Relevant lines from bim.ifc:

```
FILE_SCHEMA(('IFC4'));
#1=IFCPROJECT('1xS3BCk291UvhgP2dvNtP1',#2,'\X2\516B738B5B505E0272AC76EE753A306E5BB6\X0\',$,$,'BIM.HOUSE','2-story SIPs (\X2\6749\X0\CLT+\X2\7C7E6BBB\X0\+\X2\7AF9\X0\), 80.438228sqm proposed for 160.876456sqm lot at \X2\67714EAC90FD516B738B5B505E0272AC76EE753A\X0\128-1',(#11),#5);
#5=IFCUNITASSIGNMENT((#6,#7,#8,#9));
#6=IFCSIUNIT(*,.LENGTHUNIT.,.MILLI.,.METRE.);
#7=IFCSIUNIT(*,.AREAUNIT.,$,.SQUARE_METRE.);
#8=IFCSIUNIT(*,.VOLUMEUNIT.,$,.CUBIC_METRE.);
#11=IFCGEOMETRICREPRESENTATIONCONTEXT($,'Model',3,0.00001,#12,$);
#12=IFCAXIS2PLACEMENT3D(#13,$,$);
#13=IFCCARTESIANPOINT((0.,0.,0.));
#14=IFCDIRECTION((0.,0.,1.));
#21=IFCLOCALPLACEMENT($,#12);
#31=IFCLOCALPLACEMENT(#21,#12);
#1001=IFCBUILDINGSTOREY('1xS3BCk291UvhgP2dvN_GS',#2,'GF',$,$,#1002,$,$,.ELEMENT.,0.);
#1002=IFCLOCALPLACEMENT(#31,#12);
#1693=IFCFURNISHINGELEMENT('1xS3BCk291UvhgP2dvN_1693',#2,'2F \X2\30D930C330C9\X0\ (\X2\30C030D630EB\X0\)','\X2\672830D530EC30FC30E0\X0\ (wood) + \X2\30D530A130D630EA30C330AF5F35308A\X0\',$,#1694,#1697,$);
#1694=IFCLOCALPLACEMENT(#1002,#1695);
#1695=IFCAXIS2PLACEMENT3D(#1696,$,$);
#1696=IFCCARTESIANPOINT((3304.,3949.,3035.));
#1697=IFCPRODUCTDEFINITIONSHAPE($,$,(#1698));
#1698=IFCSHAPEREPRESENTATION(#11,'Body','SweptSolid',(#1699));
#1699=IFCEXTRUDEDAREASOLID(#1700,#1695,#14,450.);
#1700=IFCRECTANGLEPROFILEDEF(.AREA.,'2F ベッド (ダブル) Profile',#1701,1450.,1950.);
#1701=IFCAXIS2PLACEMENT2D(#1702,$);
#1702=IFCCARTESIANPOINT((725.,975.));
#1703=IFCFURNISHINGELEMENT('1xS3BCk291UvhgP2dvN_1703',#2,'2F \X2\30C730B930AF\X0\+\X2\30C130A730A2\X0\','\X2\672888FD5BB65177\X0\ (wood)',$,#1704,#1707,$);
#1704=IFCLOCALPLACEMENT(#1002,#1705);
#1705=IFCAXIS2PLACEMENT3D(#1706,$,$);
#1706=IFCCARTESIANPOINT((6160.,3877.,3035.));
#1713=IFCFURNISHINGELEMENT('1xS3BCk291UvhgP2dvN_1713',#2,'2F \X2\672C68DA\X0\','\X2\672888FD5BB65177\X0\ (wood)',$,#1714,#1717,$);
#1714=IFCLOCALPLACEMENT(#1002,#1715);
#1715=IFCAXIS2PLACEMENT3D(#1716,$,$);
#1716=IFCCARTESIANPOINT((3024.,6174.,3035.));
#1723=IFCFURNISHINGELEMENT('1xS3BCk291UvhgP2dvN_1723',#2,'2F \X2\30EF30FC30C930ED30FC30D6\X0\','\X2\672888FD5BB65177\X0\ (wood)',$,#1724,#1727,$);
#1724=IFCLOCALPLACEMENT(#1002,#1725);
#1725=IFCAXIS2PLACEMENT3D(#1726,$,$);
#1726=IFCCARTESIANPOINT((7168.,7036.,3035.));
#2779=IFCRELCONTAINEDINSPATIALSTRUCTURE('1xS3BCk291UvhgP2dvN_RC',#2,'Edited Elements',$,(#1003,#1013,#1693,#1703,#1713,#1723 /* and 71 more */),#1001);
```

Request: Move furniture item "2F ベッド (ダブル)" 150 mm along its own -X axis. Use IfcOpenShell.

```python
import ifcopenshell
import ifcopenshell.api.geometry
import ifcopenshell.util.placement

model = ifcopenshell.open("bim.ifc")

item = model.by_guid("1xS3BCk291UvhgP2dvN_1693")
matrix = ifcopenshell.util.placement.get_local_placement(item.ObjectPlacement)
matrix[:3, 3] -= matrix[:3, 0] * 150.0
ifcopenshell.api.geometry.edit_object_placement(model, product=item, matrix=matrix, is_si=False)

print(ifcopenshell.util.placement.get_local_placement(item.ObjectPlacement).round(3) + 0.0)

model.write("bim_edited.ifc")
```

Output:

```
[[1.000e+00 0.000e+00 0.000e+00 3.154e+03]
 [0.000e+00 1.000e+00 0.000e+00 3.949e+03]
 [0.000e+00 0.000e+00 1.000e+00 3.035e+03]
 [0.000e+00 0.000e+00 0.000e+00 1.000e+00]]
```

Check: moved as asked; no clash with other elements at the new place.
